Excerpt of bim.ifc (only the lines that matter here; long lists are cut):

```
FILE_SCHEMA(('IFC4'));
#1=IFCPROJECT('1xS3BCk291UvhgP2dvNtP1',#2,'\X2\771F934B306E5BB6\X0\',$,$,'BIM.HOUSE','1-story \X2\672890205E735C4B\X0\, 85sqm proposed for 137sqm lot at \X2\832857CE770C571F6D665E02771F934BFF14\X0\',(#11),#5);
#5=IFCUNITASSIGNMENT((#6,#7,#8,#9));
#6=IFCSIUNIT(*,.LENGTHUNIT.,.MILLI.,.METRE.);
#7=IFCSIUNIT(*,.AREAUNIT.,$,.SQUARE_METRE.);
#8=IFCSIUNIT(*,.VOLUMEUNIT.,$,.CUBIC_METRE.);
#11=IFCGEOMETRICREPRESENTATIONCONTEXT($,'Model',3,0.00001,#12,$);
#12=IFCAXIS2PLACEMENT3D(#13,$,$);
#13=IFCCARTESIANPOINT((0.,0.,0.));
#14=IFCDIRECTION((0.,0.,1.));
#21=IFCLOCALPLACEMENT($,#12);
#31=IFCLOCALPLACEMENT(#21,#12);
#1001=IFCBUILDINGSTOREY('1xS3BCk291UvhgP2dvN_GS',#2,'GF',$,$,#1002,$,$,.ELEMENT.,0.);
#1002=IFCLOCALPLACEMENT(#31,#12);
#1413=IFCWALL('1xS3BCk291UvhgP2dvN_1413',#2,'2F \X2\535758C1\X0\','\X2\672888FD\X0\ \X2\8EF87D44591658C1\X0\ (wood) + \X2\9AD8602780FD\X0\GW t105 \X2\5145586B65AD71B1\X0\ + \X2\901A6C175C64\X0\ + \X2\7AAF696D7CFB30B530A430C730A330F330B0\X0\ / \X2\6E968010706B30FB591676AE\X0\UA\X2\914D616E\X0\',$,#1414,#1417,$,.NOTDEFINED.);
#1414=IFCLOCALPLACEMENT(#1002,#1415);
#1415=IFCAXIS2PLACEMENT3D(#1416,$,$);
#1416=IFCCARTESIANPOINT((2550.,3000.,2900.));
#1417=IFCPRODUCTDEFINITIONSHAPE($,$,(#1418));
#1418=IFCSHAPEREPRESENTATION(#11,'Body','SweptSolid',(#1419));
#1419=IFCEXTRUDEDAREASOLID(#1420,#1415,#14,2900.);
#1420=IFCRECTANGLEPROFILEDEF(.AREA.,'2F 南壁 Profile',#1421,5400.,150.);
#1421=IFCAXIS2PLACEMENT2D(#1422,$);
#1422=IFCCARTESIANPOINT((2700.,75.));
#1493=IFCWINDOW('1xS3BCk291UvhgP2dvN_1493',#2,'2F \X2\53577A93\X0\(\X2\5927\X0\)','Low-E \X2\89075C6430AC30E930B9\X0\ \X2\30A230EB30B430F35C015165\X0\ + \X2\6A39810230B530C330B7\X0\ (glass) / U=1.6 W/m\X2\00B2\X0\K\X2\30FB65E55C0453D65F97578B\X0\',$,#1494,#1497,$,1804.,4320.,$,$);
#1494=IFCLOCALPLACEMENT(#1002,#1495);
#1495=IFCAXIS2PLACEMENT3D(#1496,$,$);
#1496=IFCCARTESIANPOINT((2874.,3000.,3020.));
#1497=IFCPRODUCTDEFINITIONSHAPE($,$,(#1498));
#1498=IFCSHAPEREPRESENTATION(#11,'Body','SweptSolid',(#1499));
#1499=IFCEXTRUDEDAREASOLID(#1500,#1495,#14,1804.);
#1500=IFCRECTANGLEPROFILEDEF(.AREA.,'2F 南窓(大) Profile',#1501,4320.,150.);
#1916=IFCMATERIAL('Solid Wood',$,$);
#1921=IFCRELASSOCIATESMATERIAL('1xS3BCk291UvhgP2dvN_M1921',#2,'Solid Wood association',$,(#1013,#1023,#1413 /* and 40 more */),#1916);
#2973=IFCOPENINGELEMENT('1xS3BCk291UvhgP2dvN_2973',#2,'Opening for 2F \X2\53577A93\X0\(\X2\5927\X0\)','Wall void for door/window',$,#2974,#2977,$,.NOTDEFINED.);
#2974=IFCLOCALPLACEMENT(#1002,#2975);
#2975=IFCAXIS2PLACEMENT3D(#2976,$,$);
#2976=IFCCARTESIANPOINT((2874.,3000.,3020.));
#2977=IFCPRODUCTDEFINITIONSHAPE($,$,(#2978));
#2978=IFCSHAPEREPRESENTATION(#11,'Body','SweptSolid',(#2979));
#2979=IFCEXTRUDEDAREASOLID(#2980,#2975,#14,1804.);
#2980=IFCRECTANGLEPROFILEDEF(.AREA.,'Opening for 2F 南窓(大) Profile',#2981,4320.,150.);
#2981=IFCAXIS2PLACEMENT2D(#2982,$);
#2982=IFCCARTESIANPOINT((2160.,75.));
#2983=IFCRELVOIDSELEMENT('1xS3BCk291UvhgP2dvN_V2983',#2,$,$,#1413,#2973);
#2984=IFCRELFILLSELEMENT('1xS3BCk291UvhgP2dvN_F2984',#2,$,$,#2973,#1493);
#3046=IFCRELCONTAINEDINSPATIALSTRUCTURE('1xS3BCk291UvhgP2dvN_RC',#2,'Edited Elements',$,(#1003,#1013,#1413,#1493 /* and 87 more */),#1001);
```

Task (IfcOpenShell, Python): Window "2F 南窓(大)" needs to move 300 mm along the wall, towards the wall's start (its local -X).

```python
import ifcopenshell
import ifcopenshell.api.geometry
import ifcopenshell.util.placement
import ifcopenshell.util.unit

model = ifcopenshell.open("bim.ifc")
unit_scale = ifcopenshell.util.unit.calculate_unit_scale(model)

window = model.by_id(1493)
opening = window.FillsVoids[0].RelatingOpeningElement
wall = opening.VoidsElements[0].RelatingBuildingElement

wall_matrix = ifcopenshell.util.placement.get_local_placement(wall.ObjectPlacement)
shift = wall_matrix[:3, 0] * -0.3 / unit_scale
before = ifcopenshell.util.placement.get_local_placement(window.ObjectPlacement)[:3, 3].copy()

# The window is not placed relative to its opening, so move both.
for product in (opening, window):
    matrix = ifcopenshell.util.placement.get_local_placement(product.ObjectPlacement)
    matrix[:3, 3] += shift
    ifcopenshell.api.geometry.edit_object_placement(model, product=product, matrix=matrix, is_si=False)

after = ifcopenshell.util.placement.get_local_placement(window.ObjectPlacement)[:3, 3]
print("window moved by", (after - before).round(3) + 0.0)

model.write("bim_updated.ifc")
```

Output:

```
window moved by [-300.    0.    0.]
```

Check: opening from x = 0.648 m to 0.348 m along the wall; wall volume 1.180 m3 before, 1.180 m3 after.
